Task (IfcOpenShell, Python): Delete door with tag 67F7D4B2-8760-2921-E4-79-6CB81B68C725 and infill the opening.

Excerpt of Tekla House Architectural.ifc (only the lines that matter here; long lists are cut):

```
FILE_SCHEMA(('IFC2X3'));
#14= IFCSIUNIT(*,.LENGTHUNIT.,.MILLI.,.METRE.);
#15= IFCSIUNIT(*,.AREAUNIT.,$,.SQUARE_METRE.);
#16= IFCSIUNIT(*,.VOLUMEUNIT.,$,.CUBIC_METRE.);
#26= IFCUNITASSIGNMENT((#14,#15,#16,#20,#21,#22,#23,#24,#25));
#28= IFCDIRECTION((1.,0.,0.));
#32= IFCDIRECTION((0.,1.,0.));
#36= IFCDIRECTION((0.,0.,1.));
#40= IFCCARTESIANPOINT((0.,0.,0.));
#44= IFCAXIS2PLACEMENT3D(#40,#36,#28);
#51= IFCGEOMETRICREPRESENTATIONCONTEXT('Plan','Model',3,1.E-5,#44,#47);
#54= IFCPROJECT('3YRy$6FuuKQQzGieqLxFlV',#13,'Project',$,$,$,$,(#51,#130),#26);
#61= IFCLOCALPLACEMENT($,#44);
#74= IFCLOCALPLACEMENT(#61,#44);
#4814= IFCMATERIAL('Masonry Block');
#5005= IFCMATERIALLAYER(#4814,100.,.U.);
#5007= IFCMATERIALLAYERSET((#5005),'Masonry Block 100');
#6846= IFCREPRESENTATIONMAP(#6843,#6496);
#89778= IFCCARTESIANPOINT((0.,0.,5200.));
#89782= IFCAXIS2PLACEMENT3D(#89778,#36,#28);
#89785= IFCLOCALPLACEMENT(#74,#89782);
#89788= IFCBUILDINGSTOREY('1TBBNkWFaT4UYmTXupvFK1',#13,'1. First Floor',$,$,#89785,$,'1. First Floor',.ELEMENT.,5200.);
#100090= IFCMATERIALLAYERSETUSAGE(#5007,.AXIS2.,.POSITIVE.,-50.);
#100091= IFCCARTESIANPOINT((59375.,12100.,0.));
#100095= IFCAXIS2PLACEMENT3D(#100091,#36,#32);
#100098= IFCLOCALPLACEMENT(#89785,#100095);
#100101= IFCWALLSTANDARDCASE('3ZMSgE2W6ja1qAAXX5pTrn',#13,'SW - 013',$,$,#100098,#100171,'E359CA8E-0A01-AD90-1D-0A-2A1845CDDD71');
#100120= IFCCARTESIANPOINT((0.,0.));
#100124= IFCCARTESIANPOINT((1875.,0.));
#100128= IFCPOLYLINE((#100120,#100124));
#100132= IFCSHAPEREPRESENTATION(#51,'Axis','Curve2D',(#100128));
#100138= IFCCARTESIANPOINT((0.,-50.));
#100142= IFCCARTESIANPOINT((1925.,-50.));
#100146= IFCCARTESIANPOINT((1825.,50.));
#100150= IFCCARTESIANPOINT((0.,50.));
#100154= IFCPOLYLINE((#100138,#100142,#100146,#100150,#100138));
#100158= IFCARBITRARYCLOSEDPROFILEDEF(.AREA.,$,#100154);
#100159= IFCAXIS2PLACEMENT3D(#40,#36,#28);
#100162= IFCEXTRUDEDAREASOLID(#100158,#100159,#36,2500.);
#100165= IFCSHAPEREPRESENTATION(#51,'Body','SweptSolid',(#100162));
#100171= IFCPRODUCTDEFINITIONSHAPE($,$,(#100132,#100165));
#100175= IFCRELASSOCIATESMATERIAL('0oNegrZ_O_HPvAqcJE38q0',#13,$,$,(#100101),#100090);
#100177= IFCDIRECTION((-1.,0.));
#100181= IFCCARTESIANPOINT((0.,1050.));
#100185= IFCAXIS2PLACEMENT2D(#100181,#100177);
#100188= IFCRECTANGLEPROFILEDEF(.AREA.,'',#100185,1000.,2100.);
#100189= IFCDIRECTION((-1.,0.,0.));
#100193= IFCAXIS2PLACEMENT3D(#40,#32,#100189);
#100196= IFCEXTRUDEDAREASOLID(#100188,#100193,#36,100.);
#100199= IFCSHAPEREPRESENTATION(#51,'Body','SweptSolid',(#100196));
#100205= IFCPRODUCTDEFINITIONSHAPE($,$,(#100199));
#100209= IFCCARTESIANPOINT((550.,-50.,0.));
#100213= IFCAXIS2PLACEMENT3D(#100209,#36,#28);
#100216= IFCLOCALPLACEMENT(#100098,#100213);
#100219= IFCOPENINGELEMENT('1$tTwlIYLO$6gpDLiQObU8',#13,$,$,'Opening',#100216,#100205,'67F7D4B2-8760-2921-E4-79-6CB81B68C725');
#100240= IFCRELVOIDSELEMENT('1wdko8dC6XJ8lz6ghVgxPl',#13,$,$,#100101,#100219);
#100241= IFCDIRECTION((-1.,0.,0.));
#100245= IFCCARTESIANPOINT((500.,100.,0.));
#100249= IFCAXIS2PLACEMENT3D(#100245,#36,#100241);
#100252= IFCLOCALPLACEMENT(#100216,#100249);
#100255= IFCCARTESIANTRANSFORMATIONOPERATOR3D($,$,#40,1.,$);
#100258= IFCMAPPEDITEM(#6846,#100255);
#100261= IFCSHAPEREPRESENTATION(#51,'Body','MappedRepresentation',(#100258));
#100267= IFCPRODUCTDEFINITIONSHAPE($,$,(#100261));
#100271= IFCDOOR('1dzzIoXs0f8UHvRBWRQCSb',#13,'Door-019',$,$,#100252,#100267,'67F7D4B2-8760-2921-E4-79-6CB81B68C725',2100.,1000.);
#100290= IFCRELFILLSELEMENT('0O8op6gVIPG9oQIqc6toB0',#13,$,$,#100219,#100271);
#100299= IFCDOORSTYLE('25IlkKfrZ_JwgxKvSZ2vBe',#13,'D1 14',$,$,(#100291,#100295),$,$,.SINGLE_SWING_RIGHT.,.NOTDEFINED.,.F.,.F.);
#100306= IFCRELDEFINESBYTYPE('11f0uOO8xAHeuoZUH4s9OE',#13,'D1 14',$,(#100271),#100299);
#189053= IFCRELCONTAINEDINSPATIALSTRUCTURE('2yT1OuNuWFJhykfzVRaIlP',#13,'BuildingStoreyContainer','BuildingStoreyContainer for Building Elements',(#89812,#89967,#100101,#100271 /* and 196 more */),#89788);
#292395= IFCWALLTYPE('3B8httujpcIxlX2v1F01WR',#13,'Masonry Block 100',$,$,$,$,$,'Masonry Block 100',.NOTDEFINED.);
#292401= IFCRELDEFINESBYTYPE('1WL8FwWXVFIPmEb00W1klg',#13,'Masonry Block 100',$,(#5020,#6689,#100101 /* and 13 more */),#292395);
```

```python
import ifcopenshell
import ifcopenshell.api.feature
import ifcopenshell.api.root
import ifcopenshell.geom
import ifcopenshell.util.shape

model = ifcopenshell.open("Tekla House Architectural.ifc")
settings = ifcopenshell.geom.settings()


def volume(element):
    """Net volume in cubic metres, openings subtracted."""
    shape = ifcopenshell.geom.create_shape(settings, element)
    return ifcopenshell.util.shape.get_volume(shape.geometry)


door = model.by_guid("1dzzIoXs0f8UHvRBWRQCSb")
opening = door.FillsVoids[0].RelatingOpeningElement
wall = opening.VoidsElements[0].RelatingBuildingElement
before = volume(wall)

ifcopenshell.api.root.remove_product(model, product=door)
ifcopenshell.api.feature.remove_feature(model, feature=opening)

after = volume(wall)

print(f"wall volume {before:.3f} -> {after:.3f} m3")

model.write("Tekla House Architectural_updated.ifc")
```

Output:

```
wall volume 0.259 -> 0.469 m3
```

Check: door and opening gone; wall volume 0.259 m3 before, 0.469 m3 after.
